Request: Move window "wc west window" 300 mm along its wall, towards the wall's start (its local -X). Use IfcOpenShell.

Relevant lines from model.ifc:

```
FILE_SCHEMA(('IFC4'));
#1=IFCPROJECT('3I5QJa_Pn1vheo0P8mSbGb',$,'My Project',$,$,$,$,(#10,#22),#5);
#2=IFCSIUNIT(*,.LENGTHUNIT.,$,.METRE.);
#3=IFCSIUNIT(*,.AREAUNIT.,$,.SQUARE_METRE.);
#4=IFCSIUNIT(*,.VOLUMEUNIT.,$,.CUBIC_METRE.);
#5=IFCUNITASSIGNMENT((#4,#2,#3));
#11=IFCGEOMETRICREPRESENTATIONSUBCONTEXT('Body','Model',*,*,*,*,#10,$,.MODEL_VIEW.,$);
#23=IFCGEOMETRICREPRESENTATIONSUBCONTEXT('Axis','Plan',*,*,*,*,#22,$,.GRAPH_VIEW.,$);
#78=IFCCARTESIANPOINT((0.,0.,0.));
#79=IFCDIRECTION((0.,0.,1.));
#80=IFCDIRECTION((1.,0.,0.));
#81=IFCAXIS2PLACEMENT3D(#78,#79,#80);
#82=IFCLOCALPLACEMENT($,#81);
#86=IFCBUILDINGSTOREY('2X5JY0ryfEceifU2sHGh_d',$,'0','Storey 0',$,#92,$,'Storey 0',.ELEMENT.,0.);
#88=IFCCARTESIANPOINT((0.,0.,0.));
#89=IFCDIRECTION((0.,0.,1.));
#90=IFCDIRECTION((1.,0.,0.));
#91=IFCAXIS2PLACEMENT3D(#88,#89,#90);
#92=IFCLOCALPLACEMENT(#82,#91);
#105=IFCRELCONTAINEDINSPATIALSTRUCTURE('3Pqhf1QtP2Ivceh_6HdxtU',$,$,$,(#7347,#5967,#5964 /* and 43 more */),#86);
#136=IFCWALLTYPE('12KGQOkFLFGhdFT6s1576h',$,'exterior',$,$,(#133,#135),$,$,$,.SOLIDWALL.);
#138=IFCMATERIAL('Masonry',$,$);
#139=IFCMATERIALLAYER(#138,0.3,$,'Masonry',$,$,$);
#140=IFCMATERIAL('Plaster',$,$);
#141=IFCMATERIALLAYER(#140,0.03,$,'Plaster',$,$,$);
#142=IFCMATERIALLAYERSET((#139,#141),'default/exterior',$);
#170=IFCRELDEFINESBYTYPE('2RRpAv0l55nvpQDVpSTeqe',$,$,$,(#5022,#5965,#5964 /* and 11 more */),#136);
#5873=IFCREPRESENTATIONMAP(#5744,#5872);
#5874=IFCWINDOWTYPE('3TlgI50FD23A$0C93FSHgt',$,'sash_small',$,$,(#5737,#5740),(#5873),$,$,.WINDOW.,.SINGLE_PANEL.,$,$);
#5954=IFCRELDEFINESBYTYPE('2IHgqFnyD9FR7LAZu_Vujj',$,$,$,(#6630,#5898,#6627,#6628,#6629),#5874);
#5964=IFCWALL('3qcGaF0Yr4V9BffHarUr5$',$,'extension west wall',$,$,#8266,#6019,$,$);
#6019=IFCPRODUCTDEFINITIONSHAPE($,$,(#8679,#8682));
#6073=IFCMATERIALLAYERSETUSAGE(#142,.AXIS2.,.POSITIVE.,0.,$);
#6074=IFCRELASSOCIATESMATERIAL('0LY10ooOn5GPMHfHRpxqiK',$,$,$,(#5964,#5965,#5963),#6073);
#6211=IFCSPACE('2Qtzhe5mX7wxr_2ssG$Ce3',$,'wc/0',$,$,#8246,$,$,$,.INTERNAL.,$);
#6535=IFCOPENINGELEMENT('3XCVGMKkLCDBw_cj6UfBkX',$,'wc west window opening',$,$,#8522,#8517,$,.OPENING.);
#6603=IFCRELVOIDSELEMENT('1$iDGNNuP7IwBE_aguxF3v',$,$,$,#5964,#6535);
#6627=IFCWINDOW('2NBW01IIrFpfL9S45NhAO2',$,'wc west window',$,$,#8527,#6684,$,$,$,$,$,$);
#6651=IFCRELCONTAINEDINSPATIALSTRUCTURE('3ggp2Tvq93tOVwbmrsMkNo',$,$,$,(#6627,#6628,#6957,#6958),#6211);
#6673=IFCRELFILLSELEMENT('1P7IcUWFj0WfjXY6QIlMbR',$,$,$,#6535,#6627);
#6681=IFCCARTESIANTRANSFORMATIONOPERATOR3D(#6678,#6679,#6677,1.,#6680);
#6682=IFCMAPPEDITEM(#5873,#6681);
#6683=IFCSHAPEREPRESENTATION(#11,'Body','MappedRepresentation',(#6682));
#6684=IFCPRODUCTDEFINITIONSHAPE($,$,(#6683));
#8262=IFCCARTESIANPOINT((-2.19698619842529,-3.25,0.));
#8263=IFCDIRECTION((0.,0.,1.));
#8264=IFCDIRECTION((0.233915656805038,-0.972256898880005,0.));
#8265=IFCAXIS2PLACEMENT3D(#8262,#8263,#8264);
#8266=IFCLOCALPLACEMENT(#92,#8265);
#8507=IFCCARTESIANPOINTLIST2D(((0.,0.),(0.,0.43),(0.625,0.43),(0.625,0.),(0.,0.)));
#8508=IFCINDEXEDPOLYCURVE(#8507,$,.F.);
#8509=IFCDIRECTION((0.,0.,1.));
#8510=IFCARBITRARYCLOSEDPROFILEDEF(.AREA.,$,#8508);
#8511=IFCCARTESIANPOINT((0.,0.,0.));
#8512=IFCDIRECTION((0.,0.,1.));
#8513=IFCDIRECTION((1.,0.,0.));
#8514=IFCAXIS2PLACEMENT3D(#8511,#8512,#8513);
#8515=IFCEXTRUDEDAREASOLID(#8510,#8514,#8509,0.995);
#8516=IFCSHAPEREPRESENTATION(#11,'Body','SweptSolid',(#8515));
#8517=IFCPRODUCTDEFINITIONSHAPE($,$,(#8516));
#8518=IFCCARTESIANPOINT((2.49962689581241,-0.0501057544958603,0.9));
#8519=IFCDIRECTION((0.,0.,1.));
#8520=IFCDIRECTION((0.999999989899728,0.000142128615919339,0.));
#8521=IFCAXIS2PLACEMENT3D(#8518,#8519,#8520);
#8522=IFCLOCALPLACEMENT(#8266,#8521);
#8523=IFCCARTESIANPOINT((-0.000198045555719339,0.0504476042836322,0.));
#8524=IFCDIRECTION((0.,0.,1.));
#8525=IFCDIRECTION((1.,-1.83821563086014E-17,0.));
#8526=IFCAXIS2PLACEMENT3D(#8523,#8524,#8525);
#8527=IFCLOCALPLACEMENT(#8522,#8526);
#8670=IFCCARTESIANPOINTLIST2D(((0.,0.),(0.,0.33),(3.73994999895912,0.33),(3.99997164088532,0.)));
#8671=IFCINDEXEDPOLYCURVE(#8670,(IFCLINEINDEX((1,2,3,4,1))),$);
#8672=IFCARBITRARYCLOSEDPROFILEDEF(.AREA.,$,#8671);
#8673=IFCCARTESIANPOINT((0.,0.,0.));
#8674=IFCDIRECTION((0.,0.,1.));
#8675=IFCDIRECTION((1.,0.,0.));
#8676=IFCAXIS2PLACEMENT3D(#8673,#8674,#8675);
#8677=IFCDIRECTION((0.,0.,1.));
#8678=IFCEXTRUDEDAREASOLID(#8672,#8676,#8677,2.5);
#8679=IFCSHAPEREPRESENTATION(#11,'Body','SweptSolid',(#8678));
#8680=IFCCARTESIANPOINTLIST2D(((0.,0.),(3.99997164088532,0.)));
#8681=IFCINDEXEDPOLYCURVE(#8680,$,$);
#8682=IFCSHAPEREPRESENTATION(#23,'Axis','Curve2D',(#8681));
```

```python
import ifcopenshell
import ifcopenshell.api.geometry
import ifcopenshell.util.placement
import ifcopenshell.util.unit

model = ifcopenshell.open("model.ifc")
unit_scale = ifcopenshell.util.unit.calculate_unit_scale(model)

window = model.by_guid("2NBW01IIrFpfL9S45NhAO2")
opening = window.FillsVoids[0].RelatingOpeningElement
wall = opening.VoidsElements[0].RelatingBuildingElement

wall_matrix = ifcopenshell.util.placement.get_local_placement(wall.ObjectPlacement)
shift = wall_matrix[:3, 0] * -0.3 / unit_scale
before = ifcopenshell.util.placement.get_local_placement(window.ObjectPlacement)[:3, 3].copy()

# The window is placed relative to its opening, so it follows when the opening moves.
matrix = ifcopenshell.util.placement.get_local_placement(opening.ObjectPlacement)
matrix[:3, 3] += shift
ifcopenshell.api.geometry.edit_object_placement(
    model, product=opening, matrix=matrix, is_si=False, should_transform_children=True
)

after = ifcopenshell.util.placement.get_local_placement(window.ObjectPlacement)[:3, 3]
print("window moved by", (after - before).round(3) + 0.0)

model.write("model_v2.ifc")
```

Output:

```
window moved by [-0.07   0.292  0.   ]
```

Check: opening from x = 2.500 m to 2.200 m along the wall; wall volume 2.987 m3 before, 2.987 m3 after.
